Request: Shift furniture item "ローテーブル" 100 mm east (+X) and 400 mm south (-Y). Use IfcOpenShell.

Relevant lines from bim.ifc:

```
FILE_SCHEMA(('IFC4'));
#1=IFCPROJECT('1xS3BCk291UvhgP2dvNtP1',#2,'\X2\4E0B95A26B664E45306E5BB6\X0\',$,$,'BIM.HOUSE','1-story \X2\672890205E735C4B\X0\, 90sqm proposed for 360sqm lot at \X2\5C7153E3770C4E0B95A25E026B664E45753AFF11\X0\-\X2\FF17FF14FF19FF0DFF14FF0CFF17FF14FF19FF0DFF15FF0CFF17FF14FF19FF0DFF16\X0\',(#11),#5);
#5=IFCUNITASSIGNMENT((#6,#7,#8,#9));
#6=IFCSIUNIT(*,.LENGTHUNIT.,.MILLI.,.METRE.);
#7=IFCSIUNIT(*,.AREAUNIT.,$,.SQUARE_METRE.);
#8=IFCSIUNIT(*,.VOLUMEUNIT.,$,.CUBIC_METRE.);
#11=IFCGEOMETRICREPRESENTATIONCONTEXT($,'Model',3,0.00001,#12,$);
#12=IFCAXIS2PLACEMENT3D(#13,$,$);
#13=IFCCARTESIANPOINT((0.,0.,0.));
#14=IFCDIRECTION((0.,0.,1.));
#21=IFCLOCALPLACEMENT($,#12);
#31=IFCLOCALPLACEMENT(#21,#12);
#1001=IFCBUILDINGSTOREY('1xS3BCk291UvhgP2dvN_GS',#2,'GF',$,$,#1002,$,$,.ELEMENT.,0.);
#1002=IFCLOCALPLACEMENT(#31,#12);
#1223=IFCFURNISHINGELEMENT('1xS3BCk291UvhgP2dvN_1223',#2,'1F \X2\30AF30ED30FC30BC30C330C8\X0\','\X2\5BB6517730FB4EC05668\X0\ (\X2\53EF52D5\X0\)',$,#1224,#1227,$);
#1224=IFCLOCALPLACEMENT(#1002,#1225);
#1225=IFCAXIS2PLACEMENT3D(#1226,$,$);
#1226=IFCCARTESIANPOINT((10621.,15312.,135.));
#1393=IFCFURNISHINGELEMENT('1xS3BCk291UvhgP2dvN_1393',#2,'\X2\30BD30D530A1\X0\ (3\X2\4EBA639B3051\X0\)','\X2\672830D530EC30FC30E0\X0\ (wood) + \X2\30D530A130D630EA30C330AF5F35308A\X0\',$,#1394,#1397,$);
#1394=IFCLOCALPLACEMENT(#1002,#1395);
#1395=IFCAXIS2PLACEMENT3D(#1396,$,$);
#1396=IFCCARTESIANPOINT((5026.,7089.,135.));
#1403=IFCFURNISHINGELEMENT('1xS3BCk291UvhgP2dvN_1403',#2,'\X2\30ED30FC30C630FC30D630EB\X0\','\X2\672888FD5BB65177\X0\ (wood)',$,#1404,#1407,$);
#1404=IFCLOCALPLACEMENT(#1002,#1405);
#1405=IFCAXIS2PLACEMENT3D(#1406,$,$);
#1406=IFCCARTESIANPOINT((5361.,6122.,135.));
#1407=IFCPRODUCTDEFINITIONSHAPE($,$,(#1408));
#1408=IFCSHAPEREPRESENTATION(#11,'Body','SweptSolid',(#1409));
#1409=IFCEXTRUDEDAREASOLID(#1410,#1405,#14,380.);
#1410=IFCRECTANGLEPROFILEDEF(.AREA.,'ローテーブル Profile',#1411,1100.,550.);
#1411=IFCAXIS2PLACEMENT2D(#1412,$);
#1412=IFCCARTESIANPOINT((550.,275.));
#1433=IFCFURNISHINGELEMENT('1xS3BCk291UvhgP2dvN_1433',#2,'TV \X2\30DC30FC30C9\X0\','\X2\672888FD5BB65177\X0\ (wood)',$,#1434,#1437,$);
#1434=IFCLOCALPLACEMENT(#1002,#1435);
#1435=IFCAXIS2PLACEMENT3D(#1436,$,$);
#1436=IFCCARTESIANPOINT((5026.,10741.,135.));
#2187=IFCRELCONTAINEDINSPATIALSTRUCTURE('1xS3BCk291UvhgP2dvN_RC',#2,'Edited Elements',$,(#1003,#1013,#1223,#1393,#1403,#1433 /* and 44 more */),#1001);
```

```python
import ifcopenshell
import ifcopenshell.api.geometry
import ifcopenshell.util.placement
import ifcopenshell.util.unit

model = ifcopenshell.open("bim.ifc")
unit_scale = ifcopenshell.util.unit.calculate_unit_scale(model)

item = model.by_guid("1xS3BCk291UvhgP2dvN_1403")
matrix = ifcopenshell.util.placement.get_local_placement(item.ObjectPlacement)
matrix[0, 3] += 0.1 / unit_scale
matrix[1, 3] -= 0.4 / unit_scale
ifcopenshell.api.geometry.edit_object_placement(model, product=item, matrix=matrix, is_si=False)

print(ifcopenshell.util.placement.get_local_placement(item.ObjectPlacement).round(3) + 0.0)

model.write("bim_edited.ifc")
```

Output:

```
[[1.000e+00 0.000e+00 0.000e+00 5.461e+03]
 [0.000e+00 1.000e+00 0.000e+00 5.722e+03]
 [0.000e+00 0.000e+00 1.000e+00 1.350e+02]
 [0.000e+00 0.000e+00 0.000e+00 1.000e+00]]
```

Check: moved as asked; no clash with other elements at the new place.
